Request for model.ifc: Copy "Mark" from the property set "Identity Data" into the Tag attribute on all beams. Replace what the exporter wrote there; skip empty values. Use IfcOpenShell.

First a look at what the model holds.

```python
import ifcopenshell
import ifcopenshell.util.element

model = ifcopenshell.open("model.ifc")
print(model.schema)
beams = model.by_type("IfcBeam")
print(len(beams), "beams")
for e in beams[:8]:
    source = ifcopenshell.util.element.get_pset(e, "Identity Data", "Mark")
    target = e.Tag
    print(e.id(), repr(source), repr(target), sep=" | ")
```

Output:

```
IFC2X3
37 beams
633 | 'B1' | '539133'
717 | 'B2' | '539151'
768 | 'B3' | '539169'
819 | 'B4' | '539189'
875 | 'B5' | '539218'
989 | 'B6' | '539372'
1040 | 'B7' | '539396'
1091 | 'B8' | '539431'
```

```python
import ifcopenshell
import ifcopenshell.util.element

model = ifcopenshell.open("model.ifc")

count = 0
for e in model.by_type("IfcBeam"):
    value = ifcopenshell.util.element.get_pset(e, "Identity Data", "Mark")
    current = e.Tag
    if not value or not value.strip() or current == value:
        continue
    e.Tag = value
    count += 1

print(count, "beams updated")

model.write("model_v2.ifc")
```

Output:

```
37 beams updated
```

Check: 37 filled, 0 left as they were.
